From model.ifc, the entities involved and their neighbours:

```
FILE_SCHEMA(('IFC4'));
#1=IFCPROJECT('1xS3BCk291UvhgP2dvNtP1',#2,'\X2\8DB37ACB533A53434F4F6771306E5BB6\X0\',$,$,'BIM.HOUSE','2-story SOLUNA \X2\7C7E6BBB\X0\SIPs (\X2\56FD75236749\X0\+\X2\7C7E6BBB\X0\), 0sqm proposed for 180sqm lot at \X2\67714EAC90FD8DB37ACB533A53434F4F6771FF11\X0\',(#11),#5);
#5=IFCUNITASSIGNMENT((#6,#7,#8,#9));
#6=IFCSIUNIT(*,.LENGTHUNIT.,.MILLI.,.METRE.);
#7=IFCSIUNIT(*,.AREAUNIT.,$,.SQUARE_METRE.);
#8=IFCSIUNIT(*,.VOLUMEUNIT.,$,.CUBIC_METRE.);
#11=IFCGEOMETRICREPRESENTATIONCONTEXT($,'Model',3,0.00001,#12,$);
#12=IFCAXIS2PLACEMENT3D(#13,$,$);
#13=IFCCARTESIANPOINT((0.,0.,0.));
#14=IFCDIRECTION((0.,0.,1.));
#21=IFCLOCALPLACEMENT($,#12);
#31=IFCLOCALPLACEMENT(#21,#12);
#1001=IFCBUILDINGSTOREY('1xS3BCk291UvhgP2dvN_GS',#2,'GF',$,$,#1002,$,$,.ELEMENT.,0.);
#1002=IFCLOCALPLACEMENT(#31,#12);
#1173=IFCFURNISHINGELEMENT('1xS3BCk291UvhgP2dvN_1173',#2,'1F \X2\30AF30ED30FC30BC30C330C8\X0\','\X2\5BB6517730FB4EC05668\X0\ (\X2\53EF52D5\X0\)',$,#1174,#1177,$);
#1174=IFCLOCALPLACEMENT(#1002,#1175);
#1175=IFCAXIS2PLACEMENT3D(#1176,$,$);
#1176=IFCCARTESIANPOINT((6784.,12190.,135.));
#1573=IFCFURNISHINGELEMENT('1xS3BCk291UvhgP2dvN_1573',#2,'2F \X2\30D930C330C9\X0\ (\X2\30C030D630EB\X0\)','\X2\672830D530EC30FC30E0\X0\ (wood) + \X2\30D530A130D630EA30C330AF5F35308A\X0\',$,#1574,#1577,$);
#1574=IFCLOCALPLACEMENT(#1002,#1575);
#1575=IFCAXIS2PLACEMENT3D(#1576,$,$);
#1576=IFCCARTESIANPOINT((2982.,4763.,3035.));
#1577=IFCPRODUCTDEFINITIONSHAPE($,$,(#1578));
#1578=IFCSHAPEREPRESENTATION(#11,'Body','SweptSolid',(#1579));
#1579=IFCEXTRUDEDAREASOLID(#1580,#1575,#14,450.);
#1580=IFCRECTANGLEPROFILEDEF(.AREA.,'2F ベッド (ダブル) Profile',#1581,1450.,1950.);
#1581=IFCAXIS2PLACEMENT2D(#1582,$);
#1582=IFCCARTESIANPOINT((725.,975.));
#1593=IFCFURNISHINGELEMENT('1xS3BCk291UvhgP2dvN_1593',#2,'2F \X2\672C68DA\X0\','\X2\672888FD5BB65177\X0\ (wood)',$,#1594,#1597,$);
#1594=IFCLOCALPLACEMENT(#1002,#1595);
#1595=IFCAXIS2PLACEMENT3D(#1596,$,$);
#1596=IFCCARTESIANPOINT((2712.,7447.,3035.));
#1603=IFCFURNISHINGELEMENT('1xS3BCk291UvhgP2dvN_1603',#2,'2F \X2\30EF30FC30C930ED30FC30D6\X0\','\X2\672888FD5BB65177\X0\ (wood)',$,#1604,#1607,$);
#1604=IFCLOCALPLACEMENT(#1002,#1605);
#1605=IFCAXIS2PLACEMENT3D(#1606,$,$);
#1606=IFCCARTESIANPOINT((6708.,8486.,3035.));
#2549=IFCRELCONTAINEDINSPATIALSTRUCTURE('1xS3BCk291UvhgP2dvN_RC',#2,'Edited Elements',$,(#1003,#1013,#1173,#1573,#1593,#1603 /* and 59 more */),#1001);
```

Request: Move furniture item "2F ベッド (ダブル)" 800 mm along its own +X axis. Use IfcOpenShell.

```python
import ifcopenshell
import ifcopenshell.api.geometry
import ifcopenshell.util.placement
import ifcopenshell.util.unit

model = ifcopenshell.open("model.ifc")
unit_scale = ifcopenshell.util.unit.calculate_unit_scale(model)

item = model.by_guid("1xS3BCk291UvhgP2dvN_1573")
matrix = ifcopenshell.util.placement.get_local_placement(item.ObjectPlacement)
matrix[:3, 3] += matrix[:3, 0] * 0.8 / unit_scale
ifcopenshell.api.geometry.edit_object_placement(model, product=item, matrix=matrix, is_si=False)

print(ifcopenshell.util.placement.get_local_placement(item.ObjectPlacement).round(3) + 0.0)

model.write("model_updated.ifc")
```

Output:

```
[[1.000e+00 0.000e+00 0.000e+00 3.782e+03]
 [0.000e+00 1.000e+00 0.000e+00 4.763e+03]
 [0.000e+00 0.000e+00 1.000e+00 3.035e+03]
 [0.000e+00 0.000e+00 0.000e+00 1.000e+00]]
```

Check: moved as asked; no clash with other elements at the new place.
